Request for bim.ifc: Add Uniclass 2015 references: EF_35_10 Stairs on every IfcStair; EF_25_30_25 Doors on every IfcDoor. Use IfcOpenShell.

First a look at what the model holds.

```python
import ifcopenshell

model = ifcopenshell.open("bim.ifc")
print(model.schema)
print("classifications:", [c.Name for c in model.by_type("IfcClassification")])
for ifc_class in ("IfcDoor", "IfcRoof", "IfcStair", "IfcWall", "IfcWindow"):
    print(ifc_class, len(model.by_type(ifc_class)))
```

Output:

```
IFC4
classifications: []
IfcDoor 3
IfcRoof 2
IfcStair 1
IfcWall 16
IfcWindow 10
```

```python
import ifcopenshell
import ifcopenshell.api.classification

model = ifcopenshell.open("bim.ifc")

system = ifcopenshell.api.classification.add_classification(model, classification="Uniclass 2015")

codes = {
    "IfcStair": ("EF_35_10", "Stairs"),
    "IfcDoor": ("EF_25_30_25", "Doors"),
}
for ifc_class, (code, name) in codes.items():
    products = model.by_type(ifc_class)
    ifcopenshell.api.classification.add_reference(
        model, products=products, classification=system, identification=code, name=name
    )
    print(code, len(products))

model.write("bim-out.ifc")
```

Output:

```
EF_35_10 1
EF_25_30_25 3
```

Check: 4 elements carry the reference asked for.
